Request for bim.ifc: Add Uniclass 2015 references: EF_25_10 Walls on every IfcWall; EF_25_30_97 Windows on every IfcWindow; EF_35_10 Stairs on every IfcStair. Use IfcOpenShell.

First a look at what the model holds.

```python
import ifcopenshell

model = ifcopenshell.open("bim.ifc")
print(model.schema)
print("classifications:", [c.Name for c in model.by_type("IfcClassification")])
for ifc_class in ("IfcDoor", "IfcRoof", "IfcStair", "IfcWall", "IfcWindow"):
    print(ifc_class, len(model.by_type(ifc_class)))
```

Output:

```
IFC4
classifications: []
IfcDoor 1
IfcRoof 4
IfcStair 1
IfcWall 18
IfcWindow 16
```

```python
import ifcopenshell
import ifcopenshell.api.classification

model = ifcopenshell.open("bim.ifc")

system = ifcopenshell.api.classification.add_classification(model, classification="Uniclass 2015")

codes = {
    "IfcWall": ("EF_25_10", "Walls"),
    "IfcWindow": ("EF_25_30_97", "Windows"),
    "IfcStair": ("EF_35_10", "Stairs"),
}
for ifc_class, (code, name) in codes.items():
    products = model.by_type(ifc_class)
    ifcopenshell.api.classification.add_reference(
        model, products=products, classification=system, identification=code, name=name
    )
    print(code, len(products))

model.write("bim-out.ifc")
```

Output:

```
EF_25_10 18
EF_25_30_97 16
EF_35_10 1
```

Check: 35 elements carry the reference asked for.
